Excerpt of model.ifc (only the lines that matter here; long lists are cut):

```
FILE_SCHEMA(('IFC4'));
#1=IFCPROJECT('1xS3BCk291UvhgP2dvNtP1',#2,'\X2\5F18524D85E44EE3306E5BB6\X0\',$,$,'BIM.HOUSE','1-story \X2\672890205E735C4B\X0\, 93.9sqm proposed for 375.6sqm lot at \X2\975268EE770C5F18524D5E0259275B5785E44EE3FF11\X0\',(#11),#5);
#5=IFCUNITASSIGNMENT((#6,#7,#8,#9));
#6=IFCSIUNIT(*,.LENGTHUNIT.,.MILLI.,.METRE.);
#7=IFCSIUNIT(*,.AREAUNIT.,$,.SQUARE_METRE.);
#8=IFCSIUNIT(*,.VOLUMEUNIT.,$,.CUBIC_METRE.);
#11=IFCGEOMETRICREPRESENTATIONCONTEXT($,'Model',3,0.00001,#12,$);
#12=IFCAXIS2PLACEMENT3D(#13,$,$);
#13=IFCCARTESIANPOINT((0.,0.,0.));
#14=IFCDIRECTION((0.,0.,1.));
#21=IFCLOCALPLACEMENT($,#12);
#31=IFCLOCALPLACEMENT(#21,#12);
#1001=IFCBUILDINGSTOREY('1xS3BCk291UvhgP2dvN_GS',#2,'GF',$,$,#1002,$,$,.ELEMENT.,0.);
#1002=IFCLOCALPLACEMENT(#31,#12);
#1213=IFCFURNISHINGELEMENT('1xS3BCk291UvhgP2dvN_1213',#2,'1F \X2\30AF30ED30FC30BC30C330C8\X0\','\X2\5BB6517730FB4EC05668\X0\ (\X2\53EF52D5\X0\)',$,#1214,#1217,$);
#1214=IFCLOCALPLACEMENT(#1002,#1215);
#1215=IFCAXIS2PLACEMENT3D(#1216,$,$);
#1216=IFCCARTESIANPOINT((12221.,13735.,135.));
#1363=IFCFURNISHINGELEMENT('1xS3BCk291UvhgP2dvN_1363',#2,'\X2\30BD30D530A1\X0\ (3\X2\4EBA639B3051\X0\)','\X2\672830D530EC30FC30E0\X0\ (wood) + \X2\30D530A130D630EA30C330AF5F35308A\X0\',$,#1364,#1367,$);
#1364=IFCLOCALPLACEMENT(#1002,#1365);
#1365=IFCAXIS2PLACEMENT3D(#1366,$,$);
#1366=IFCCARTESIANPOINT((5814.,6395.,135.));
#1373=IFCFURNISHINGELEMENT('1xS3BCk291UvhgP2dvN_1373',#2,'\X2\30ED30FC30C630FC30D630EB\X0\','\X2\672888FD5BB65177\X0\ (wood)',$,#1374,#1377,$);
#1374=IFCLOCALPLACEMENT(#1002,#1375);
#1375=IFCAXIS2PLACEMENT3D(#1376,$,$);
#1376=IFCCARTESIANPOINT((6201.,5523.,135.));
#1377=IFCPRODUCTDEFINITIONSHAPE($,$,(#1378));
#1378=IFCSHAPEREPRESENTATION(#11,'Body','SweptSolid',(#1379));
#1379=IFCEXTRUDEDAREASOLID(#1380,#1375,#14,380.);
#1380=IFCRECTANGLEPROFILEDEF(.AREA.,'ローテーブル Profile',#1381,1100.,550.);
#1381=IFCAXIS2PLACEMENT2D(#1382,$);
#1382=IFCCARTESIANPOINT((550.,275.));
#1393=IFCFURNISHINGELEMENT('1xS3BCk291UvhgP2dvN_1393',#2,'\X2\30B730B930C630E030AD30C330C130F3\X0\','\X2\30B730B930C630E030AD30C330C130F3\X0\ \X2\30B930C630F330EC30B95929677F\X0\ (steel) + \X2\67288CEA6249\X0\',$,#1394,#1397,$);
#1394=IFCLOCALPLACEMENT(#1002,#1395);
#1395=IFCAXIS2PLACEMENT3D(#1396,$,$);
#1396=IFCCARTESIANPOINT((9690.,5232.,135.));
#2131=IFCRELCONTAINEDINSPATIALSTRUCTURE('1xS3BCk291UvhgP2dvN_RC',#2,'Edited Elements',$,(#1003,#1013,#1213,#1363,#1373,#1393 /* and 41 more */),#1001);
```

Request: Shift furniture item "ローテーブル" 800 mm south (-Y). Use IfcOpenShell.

```python
import ifcopenshell
import ifcopenshell.api.geometry
import ifcopenshell.util.placement

model = ifcopenshell.open("model.ifc")

item = model.by_guid("1xS3BCk291UvhgP2dvN_1373")
matrix = ifcopenshell.util.placement.get_local_placement(item.ObjectPlacement)
matrix[1, 3] -= 800.0
ifcopenshell.api.geometry.edit_object_placement(model, product=item, matrix=matrix, is_si=False)

print(ifcopenshell.util.placement.get_local_placement(item.ObjectPlacement).round(3) + 0.0)

model.write("model-out.ifc")
```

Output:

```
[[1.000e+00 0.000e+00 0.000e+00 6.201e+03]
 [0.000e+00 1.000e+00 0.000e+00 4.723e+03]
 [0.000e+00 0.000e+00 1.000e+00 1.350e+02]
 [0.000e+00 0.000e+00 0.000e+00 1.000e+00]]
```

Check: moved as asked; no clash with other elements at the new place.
